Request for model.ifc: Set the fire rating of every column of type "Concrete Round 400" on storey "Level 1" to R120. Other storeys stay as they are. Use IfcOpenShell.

First a look at what the model holds.

```python
import ifcopenshell
import ifcopenshell.util.element

model = ifcopenshell.open("model.ifc")
print(model.schema)
storey = next(s for s in model.by_type("IfcBuildingStorey") if s.Name == "Level 1")
columns = [e for e in ifcopenshell.util.element.get_decomposition(storey) if e.is_a("IfcColumn")]
seen = {}
for e in columns:
    element_type = ifcopenshell.util.element.get_type(e)
    key = (element_type.Name if element_type != e and element_type else None, ifcopenshell.util.element.get_pset(e, "Pset_ColumnCommon", "FireRating"))
    seen[key] = seen.get(key, 0) + 1
for (name, value), count in sorted(seen.items(), key=str):
    print(count, "x", name, "|", value)
```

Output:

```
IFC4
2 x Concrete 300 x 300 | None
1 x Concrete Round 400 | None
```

```python
import ifcopenshell
import ifcopenshell.api.pset
import ifcopenshell.util.element

model = ifcopenshell.open("model.ifc")

storey = next(s for s in model.by_type("IfcBuildingStorey") if s.Name == "Level 1")
columns = [e for e in ifcopenshell.util.element.get_decomposition(storey) if e.is_a("IfcColumn")]

count = 0
for e in columns:
    element_type = ifcopenshell.util.element.get_type(e)
    if element_type in (None, e) or element_type.Name != "Concrete Round 400":
        continue
    # add_pset returns the element's existing set when there is one.
    pset = ifcopenshell.api.pset.add_pset(model, product=e, name="Pset_ColumnCommon")
    ifcopenshell.api.pset.edit_pset(model, pset=pset, properties={"FireRating": "R120"})
    count += 1

print(count, "columns updated")

model.write("model_edited.ifc")
```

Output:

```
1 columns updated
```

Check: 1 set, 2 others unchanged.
